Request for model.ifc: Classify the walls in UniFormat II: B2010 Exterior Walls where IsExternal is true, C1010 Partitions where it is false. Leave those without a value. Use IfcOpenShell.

First a look at what the model holds.

```python
import ifcopenshell
import ifcopenshell.util.element

model = ifcopenshell.open("model.ifc")
print(model.schema)
print("classifications:", [c.Name for c in model.by_type("IfcClassification")])
values = [ifcopenshell.util.element.get_pset(e, "Pset_WallCommon", "IsExternal") for e in model.by_type("IfcWall")]
for value in (True, False, None):
    print("IsExternal", value, values.count(value))
```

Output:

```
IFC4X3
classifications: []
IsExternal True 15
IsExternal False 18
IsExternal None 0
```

```python
import ifcopenshell
import ifcopenshell.api.classification
import ifcopenshell.util.element

model = ifcopenshell.open("model.ifc")

system = ifcopenshell.api.classification.add_classification(model, classification="UniFormat II")

walls = model.by_type("IfcWall")
external = {e: ifcopenshell.util.element.get_pset(e, "Pset_WallCommon", "IsExternal") for e in walls}
for flag, code, name in ((True, "B2010", "Exterior Walls"), (False, "C1010", "Partitions")):
    products = [e for e in walls if external[e] is flag]
    ifcopenshell.api.classification.add_reference(
        model, products=products, classification=system, identification=code, name=name
    )
    print(code, len(products))

model.write("model-out.ifc")
```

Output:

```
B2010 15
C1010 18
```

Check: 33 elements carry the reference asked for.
